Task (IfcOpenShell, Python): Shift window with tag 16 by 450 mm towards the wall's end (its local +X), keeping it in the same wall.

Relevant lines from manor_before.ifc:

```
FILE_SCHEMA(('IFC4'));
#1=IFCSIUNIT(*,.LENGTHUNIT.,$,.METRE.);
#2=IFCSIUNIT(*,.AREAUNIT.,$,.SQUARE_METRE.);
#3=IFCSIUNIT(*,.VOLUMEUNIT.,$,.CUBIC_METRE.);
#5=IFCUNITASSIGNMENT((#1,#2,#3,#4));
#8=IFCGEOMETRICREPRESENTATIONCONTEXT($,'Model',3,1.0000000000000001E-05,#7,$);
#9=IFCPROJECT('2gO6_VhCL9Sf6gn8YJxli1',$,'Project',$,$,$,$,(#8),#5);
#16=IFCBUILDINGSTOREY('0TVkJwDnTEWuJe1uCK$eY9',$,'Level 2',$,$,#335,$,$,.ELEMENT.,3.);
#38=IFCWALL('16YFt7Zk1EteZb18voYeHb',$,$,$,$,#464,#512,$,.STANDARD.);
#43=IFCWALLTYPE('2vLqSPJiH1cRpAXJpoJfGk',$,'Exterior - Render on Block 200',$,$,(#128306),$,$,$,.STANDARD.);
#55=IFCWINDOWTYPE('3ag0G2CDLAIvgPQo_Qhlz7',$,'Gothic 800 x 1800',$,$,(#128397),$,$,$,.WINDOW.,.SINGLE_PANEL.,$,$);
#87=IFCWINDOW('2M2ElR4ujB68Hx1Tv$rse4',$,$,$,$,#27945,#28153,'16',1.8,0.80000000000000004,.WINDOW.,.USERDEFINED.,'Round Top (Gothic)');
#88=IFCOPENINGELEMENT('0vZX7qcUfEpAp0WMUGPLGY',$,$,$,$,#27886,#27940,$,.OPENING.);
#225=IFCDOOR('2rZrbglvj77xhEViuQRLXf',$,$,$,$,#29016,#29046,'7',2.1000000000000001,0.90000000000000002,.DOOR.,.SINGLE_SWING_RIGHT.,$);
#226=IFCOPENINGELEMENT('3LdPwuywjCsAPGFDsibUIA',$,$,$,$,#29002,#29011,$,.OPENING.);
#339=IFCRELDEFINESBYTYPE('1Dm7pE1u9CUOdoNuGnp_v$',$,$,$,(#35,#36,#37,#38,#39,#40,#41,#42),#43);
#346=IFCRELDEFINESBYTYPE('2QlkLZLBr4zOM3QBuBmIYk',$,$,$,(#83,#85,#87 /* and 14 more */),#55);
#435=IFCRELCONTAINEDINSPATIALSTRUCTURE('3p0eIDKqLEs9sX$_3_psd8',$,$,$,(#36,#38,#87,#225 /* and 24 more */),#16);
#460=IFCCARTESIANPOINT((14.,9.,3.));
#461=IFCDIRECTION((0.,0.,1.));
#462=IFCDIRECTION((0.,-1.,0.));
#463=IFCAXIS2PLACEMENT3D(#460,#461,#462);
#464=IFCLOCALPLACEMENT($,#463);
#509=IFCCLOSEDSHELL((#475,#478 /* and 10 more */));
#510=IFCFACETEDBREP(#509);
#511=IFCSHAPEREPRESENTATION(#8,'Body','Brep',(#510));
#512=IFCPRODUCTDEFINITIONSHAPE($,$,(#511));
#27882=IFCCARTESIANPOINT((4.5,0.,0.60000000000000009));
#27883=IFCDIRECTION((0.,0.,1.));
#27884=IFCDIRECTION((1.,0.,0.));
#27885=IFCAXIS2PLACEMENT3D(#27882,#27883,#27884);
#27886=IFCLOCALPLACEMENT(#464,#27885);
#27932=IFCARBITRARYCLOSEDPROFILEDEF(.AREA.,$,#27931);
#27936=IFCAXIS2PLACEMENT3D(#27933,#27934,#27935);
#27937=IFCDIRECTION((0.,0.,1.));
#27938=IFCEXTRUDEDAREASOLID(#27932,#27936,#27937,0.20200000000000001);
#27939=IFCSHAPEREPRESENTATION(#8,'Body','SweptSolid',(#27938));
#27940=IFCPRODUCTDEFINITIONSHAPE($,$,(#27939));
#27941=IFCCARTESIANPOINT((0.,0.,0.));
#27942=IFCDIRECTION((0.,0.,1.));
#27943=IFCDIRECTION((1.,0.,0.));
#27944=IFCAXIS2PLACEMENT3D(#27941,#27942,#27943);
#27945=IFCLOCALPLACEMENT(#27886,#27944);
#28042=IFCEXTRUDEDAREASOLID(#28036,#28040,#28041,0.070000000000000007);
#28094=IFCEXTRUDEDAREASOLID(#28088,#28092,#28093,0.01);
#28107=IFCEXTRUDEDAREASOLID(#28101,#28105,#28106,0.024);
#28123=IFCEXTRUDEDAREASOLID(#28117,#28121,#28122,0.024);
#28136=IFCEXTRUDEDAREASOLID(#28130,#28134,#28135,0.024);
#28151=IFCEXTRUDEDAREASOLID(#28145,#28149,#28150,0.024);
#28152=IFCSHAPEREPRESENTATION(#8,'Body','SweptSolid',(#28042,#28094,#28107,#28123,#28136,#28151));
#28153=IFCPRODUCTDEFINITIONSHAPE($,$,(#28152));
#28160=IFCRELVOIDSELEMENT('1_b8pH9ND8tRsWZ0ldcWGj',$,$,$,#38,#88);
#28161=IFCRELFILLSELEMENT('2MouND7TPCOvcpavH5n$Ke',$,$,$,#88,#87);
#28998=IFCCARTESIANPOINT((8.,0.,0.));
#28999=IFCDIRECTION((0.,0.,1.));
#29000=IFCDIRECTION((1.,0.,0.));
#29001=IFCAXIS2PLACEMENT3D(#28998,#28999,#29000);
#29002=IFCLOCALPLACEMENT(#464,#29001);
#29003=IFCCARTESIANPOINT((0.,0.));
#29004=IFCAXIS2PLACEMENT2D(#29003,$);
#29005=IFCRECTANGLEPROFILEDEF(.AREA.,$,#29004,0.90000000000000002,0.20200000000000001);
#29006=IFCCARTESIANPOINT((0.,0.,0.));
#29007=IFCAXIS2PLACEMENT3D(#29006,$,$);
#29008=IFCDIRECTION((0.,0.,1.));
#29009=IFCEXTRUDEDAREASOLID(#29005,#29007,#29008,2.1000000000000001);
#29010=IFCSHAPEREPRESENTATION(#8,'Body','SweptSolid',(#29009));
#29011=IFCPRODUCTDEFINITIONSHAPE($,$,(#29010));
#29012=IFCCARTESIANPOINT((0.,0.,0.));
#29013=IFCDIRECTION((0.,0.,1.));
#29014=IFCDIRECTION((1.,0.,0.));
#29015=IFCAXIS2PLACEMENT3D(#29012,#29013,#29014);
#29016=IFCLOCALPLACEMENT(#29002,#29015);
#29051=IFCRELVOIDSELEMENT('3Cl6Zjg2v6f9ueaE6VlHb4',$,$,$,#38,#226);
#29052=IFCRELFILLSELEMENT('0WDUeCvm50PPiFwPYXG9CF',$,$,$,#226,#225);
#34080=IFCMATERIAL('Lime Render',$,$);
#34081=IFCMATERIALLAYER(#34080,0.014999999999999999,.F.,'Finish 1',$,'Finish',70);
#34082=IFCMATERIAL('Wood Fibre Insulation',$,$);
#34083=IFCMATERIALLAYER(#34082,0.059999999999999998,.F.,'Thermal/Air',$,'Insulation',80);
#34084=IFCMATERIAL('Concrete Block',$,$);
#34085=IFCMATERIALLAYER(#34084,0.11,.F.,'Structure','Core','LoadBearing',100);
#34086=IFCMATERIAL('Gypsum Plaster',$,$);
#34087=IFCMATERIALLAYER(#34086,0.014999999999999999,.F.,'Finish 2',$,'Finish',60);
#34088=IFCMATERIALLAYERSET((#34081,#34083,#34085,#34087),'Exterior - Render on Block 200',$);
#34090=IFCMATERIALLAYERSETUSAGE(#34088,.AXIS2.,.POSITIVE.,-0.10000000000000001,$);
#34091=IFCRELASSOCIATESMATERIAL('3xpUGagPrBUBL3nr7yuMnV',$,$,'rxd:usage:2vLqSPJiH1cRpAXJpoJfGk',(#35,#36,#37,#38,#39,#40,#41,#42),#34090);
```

```python
import ifcopenshell
import ifcopenshell.api.geometry
import ifcopenshell.util.placement
import ifcopenshell.util.unit

model = ifcopenshell.open("manor_before.ifc")
unit_scale = ifcopenshell.util.unit.calculate_unit_scale(model)

window = model.by_guid("2M2ElR4ujB68Hx1Tv$rse4")
opening = window.FillsVoids[0].RelatingOpeningElement
wall = opening.VoidsElements[0].RelatingBuildingElement

wall_matrix = ifcopenshell.util.placement.get_local_placement(wall.ObjectPlacement)
shift = wall_matrix[:3, 0] * 0.45 / unit_scale
before = ifcopenshell.util.placement.get_local_placement(window.ObjectPlacement)[:3, 3].copy()

# The window is placed relative to its opening, so it follows when the opening moves.
matrix = ifcopenshell.util.placement.get_local_placement(opening.ObjectPlacement)
matrix[:3, 3] += shift
ifcopenshell.api.geometry.edit_object_placement(
    model, product=opening, matrix=matrix, is_si=False, should_transform_children=True
)

after = ifcopenshell.util.placement.get_local_placement(window.ObjectPlacement)[:3, 3]
print("window moved by", (after - before).round(3) + 0.0)

model.write("manor_before_v2.ifc")
```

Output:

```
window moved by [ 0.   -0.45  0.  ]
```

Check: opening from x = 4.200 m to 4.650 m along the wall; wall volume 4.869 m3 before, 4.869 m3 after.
